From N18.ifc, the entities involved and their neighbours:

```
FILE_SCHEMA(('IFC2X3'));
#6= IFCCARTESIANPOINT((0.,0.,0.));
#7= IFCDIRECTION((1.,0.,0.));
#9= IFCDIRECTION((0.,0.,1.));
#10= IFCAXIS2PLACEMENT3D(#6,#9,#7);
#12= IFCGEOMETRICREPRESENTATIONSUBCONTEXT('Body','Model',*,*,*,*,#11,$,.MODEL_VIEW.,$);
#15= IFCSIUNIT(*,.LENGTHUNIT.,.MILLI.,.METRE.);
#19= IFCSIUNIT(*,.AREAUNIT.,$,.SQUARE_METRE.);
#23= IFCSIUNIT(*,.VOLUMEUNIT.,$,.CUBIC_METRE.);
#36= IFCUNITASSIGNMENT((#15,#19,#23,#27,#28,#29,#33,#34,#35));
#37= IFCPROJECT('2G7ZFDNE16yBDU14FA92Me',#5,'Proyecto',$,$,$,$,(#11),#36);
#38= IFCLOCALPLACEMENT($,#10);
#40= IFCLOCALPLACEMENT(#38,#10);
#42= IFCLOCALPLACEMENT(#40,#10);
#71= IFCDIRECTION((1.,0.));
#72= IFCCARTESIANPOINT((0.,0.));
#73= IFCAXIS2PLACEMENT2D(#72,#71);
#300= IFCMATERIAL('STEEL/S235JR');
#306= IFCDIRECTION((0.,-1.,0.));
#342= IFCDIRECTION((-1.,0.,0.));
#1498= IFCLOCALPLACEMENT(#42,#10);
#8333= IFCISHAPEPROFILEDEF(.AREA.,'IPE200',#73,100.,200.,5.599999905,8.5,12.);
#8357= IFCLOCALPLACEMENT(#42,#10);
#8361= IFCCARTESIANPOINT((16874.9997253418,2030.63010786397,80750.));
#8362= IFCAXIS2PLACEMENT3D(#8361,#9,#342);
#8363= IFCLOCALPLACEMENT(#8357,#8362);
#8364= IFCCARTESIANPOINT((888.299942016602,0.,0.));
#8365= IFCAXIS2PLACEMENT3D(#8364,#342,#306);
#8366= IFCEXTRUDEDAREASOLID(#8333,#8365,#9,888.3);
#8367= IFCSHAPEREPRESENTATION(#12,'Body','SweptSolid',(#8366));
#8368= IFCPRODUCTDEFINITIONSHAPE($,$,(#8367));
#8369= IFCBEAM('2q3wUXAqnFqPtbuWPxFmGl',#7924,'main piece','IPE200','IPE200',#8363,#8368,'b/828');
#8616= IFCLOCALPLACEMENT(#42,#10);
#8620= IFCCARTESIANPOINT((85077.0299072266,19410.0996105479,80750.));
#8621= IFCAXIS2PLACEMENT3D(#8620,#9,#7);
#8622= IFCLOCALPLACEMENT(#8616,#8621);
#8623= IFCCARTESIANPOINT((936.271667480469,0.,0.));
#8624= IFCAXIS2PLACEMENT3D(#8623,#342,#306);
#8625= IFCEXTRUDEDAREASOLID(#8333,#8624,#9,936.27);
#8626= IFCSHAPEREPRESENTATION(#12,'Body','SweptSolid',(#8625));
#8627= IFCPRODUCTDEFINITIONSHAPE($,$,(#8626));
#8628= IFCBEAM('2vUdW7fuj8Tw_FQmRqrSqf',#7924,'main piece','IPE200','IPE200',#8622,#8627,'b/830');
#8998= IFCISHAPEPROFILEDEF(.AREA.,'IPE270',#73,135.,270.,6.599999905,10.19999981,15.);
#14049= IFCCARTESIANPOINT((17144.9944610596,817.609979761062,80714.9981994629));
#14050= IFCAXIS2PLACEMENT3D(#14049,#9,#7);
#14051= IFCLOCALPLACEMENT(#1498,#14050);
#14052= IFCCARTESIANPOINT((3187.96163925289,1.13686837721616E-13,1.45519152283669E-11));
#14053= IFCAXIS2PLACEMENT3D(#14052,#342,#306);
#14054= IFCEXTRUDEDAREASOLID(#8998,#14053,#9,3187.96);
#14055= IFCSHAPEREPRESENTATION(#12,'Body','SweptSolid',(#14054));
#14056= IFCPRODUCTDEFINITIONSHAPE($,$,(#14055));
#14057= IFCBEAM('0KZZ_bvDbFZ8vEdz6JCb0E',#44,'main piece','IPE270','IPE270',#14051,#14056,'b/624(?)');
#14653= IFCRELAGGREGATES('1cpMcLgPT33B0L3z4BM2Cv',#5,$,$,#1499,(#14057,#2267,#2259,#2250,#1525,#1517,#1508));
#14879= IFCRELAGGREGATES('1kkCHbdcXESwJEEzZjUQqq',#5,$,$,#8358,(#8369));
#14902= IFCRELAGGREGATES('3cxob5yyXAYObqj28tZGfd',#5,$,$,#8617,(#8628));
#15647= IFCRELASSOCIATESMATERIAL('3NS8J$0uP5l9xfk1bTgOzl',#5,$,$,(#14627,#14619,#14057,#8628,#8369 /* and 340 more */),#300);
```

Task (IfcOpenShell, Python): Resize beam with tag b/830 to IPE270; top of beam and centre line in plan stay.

```python
import ifcopenshell
import ifcopenshell.util.element
import ifcopenshell.util.representation

model = ifcopenshell.open("N18.ifc")

member = model.by_guid("2vUdW7fuj8Tw_FQmRqrSqf")
source = next(p for p in model.by_type("IfcIShapeProfileDef") if p.ProfileName == "IPE270")

body = ifcopenshell.util.representation.get_representation(member, "Model", "Body")
solid = body.Items[0]
old_profile = solid.SweptArea

# Copy the section's sizes but keep this member's own profile position.
profile = ifcopenshell.util.element.copy(model, source)
# Profiles are centred, so shift by half the change in depth to hold the top.
shift = (old_profile.OverallDepth - profile.OverallDepth) / 2
x, y = old_profile.Position.Location.Coordinates
up = (0.0, 1.0)  # upwards, in the solid's own plane
location = model.createIfcCartesianPoint((x + up[0] * shift, y + up[1] * shift))
profile.Position = model.createIfcAxis2Placement2D(location, old_profile.Position.RefDirection)
solid.SweptArea = profile
if not model.get_total_inverses(old_profile):
    ifcopenshell.util.element.remove_deep2(model, old_profile)
member.Description = member.Description.replace("IPE200", "IPE270")
member.ObjectType = member.ObjectType.replace("IPE200", "IPE270")

print(solid.SweptArea)

model.write("N18-out.ifc")
```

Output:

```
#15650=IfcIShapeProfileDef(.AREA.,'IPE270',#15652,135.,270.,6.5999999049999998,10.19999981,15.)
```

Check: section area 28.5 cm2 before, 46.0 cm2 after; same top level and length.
